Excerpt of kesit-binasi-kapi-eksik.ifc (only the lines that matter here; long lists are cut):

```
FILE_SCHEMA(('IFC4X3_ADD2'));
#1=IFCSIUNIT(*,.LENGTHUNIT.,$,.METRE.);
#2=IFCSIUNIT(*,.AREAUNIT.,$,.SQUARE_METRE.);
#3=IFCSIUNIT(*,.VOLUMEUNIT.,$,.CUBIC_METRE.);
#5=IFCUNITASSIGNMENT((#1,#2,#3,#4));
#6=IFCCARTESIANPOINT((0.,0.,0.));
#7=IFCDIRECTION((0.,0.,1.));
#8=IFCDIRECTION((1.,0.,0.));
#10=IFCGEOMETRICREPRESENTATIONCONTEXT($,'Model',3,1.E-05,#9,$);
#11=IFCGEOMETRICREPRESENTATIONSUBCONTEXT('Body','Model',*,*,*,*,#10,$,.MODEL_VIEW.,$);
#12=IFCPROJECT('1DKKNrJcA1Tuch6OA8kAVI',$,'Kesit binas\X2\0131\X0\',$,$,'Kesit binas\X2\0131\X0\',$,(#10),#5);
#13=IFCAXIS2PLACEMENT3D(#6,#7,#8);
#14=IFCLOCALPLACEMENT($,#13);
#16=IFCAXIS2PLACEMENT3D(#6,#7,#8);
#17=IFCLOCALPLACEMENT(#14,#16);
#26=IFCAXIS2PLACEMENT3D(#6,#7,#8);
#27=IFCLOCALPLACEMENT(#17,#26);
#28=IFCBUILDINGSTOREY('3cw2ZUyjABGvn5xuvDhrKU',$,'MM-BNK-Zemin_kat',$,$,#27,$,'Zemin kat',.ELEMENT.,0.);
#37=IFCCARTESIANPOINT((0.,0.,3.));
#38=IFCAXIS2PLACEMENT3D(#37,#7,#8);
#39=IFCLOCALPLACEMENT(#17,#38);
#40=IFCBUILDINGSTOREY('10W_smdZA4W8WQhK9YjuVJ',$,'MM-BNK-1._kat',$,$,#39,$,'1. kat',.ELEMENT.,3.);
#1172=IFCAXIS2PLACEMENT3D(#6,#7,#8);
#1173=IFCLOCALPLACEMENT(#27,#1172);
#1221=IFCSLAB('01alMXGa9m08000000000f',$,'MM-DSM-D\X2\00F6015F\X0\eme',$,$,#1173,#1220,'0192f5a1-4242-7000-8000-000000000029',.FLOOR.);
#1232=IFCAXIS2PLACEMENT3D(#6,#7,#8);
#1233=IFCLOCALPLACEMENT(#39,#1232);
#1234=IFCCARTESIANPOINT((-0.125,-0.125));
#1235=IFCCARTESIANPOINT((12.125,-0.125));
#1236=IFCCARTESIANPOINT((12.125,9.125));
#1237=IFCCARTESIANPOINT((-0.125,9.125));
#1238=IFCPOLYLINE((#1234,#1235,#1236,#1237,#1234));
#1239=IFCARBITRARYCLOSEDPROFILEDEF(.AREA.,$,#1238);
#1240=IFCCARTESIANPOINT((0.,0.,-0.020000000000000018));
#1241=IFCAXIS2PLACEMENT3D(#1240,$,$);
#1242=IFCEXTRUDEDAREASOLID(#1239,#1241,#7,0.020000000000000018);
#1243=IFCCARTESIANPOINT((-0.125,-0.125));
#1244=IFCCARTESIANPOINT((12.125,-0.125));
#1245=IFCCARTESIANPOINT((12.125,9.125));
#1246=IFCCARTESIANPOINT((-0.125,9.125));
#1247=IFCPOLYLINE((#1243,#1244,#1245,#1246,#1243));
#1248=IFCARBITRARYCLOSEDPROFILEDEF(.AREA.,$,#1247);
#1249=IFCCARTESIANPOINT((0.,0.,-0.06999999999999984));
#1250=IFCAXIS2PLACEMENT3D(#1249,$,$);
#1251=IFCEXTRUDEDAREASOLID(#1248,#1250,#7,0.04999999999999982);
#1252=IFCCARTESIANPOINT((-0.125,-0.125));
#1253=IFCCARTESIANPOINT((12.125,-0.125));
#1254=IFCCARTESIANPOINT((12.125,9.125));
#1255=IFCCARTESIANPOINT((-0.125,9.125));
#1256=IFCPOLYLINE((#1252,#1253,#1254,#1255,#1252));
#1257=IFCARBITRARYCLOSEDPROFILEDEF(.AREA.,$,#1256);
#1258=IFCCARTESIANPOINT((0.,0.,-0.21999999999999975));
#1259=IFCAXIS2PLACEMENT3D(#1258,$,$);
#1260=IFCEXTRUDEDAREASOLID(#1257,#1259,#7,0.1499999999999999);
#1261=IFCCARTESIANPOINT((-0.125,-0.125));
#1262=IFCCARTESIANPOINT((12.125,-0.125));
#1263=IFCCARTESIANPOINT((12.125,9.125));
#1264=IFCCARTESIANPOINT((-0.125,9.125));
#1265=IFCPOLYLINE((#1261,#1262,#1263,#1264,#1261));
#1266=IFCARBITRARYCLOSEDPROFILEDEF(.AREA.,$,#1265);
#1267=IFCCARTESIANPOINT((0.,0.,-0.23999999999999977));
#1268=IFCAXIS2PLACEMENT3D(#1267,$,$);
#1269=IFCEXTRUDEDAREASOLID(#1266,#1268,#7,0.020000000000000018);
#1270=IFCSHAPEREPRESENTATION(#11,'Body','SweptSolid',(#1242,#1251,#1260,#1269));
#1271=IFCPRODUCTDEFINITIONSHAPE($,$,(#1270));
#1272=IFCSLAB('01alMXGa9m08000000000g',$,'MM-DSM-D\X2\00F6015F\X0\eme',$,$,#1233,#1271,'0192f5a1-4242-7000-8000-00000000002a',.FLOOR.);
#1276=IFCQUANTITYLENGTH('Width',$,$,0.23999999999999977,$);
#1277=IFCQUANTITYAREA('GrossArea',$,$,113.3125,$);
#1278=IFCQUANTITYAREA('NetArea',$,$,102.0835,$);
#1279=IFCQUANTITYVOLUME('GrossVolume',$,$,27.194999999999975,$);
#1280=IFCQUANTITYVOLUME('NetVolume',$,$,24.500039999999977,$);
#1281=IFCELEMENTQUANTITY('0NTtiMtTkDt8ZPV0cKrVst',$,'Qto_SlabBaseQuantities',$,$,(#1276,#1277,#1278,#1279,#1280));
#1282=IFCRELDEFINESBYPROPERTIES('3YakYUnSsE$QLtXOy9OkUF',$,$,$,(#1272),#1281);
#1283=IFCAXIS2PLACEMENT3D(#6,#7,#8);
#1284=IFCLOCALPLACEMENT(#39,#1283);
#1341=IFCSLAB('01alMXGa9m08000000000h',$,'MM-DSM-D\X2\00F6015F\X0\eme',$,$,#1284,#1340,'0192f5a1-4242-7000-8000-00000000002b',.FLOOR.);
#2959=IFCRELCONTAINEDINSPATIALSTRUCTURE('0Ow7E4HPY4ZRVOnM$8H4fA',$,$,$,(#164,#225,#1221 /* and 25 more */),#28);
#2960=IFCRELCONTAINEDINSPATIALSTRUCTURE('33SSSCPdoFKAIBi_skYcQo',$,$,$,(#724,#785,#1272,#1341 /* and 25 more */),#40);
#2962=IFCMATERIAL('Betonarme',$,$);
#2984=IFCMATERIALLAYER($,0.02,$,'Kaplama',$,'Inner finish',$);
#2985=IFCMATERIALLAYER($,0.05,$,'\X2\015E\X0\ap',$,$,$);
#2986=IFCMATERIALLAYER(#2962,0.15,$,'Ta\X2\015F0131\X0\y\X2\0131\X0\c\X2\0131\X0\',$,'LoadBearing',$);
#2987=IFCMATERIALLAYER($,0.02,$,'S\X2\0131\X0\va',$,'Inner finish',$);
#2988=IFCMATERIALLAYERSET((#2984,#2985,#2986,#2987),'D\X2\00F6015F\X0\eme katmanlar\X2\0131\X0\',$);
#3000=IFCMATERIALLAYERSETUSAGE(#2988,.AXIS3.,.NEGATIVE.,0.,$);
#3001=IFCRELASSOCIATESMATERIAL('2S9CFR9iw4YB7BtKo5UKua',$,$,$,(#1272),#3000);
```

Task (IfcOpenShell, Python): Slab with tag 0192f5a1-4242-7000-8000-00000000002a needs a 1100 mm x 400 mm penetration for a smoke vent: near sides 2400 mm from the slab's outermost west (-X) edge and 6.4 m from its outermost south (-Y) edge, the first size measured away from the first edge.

```python
import numpy as np
import ifcopenshell
import ifcopenshell.api.feature
import ifcopenshell.api.geometry
import ifcopenshell.api.pset
import ifcopenshell.api.root
import ifcopenshell.geom
import ifcopenshell.util.element
import ifcopenshell.util.placement
import ifcopenshell.util.representation
import ifcopenshell.util.shape
import ifcopenshell.util.unit

model = ifcopenshell.open("kesit-binasi-kapi-eksik.ifc")
unit_scale = ifcopenshell.util.unit.calculate_unit_scale(model)
area_scale = ifcopenshell.util.unit.calculate_unit_scale(model, "AREAUNIT")
volume_scale = ifcopenshell.util.unit.calculate_unit_scale(model, "VOLUMEUNIT")
settings = ifcopenshell.geom.settings()


def volume(element):
    """Net volume in cubic metres, openings subtracted."""
    shape = ifcopenshell.geom.create_shape(settings, element)
    return ifcopenshell.util.shape.get_volume(shape.geometry)


slab = model.by_guid("01alMXGa9m08000000000g")
before = volume(slab)

# Extent in the slab's own axes, in metres. The edges named are its -X and -Y sides.
slab_shape = ifcopenshell.geom.create_shape(settings, slab)
vertices = ifcopenshell.util.shape.get_vertices(slab_shape.geometry)
x_min, y_min, bottom = vertices.min(axis=0)
top = vertices[:, 2].max()

opening = ifcopenshell.api.root.create_entity(model, ifc_class="IfcOpeningElement", name="Smoke vent opening", predefined_type="OPENING")
context = ifcopenshell.util.representation.get_context(model, "Model", "Body", "MODEL_VIEW")
width, depth = 1.1, 0.4
outline = [(0.0, 0.0), (width, 0.0), (width, depth), (0.0, depth), (0.0, 0.0)]
# Overshoot both faces by 50 mm so the cut is clean.
shape = ifcopenshell.api.geometry.add_slab_representation(
    model, context=context, depth=top - bottom + 0.1, polyline=outline
)
ifcopenshell.api.geometry.assign_representation(model, product=opening, representation=shape)

matrix = ifcopenshell.util.placement.get_local_placement(slab.ObjectPlacement)
matrix[:, 3] = matrix @ np.append(np.array([x_min + 2.4, y_min + 6.4, bottom - 0.05]) / unit_scale, 1.0)
ifcopenshell.api.geometry.edit_object_placement(model, product=opening, matrix=matrix, is_si=False)
ifcopenshell.api.feature.add_feature(model, feature=opening, element=slab)

after = volume(slab)

# Update the slab's stored quantities.
qto = model.by_id(ifcopenshell.util.element.get_pset(slab, "Qto_SlabBaseQuantities", should_inherit=False)["id"])
ifcopenshell.api.pset.edit_qto(model, qto=qto, properties={
    "NetArea": after / (top - bottom) / area_scale,
    "NetVolume": after / volume_scale,
})

print(f"slab volume {before:.3f} -> {after:.3f} m3")

model.write("kesit-binasi-kapi-eksik_updated.ifc")
```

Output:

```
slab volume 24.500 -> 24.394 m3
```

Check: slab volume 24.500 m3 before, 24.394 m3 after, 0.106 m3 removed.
